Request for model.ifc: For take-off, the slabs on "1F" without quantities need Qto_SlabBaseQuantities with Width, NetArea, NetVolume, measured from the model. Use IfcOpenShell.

First a look at what the model holds.

```python
import ifcopenshell
import ifcopenshell.util.element
import ifcopenshell.util.unit

model = ifcopenshell.open("model.ifc")
print(model.schema)
for unit_type in ("LENGTHUNIT", "AREAUNIT", "VOLUMEUNIT"):
    print(unit_type, ifcopenshell.util.unit.calculate_unit_scale(model, unit_type))
storey = next(s for s in model.by_type("IfcBuildingStorey") if s.Name == "1F")
slabs = [e for e in ifcopenshell.util.element.get_decomposition(storey) if e.is_a("IfcSlab")]
for e in sorted(slabs, key=lambda e: e.id()):
    print(e.id(), e.is_a(), e.Name, list(ifcopenshell.util.element.get_psets(e, qtos_only=True)), sep=" | ")
```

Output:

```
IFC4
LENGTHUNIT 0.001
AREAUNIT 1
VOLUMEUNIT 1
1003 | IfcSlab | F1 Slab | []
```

```python
import ifcopenshell
import ifcopenshell.api.pset
import ifcopenshell.geom
import ifcopenshell.util.element
import ifcopenshell.util.shape
import ifcopenshell.util.unit

model = ifcopenshell.open("model.ifc")
unit_scale = ifcopenshell.util.unit.calculate_unit_scale(model)
area_scale = ifcopenshell.util.unit.calculate_unit_scale(model, "AREAUNIT")
volume_scale = ifcopenshell.util.unit.calculate_unit_scale(model, "VOLUMEUNIT")
settings = ifcopenshell.geom.settings()

storey = next(s for s in model.by_type("IfcBuildingStorey") if s.Name == "1F")
slabs = [e for e in ifcopenshell.util.element.get_decomposition(storey) if e.is_a("IfcSlab")]

for e in sorted(slabs, key=lambda e: e.id()):
    if ifcopenshell.util.element.get_psets(e, qtos_only=True, should_inherit=False):
        continue
    # Geometry comes back in metres, in the element's own axes.
    shape = ifcopenshell.geom.create_shape(settings, e)
    values = {
        "Width": ifcopenshell.util.shape.get_z(shape.geometry) / unit_scale,
        "NetArea": ifcopenshell.util.shape.get_footprint_area(shape.geometry) / area_scale,
        "NetVolume": ifcopenshell.util.shape.get_volume(shape.geometry) / volume_scale,
    }
    qto = ifcopenshell.api.pset.add_qto(model, product=e, name="Qto_SlabBaseQuantities")
    ifcopenshell.api.pset.edit_qto(model, qto=qto, properties=values)
    print(e.id(), {k: round(v, 3) for k, v in values.items()})

model.write("model-out.ifc")
```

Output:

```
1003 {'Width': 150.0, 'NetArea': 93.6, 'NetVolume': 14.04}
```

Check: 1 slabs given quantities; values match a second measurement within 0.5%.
